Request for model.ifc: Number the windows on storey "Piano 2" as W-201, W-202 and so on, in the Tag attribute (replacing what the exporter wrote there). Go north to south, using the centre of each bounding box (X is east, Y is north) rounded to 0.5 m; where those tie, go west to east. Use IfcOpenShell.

First a look at what the model holds.

```python
import ifcopenshell
import ifcopenshell.util.element
import ifcopenshell.util.placement

model = ifcopenshell.open("model.ifc")
print(model.schema)
storey = next(s for s in model.by_type("IfcBuildingStorey") if s.Name == "Piano 2")
windows = [e for e in ifcopenshell.util.element.get_decomposition(storey) if e.is_a("IfcWindow")]
for e in sorted(windows, key=lambda e: e.id()):
    origin = ifcopenshell.util.placement.get_local_placement(e.ObjectPlacement)[:3, 3]
    print(e.id(), e.Tag, e.Name, origin.round(2) + 0.0, sep=" | ")
```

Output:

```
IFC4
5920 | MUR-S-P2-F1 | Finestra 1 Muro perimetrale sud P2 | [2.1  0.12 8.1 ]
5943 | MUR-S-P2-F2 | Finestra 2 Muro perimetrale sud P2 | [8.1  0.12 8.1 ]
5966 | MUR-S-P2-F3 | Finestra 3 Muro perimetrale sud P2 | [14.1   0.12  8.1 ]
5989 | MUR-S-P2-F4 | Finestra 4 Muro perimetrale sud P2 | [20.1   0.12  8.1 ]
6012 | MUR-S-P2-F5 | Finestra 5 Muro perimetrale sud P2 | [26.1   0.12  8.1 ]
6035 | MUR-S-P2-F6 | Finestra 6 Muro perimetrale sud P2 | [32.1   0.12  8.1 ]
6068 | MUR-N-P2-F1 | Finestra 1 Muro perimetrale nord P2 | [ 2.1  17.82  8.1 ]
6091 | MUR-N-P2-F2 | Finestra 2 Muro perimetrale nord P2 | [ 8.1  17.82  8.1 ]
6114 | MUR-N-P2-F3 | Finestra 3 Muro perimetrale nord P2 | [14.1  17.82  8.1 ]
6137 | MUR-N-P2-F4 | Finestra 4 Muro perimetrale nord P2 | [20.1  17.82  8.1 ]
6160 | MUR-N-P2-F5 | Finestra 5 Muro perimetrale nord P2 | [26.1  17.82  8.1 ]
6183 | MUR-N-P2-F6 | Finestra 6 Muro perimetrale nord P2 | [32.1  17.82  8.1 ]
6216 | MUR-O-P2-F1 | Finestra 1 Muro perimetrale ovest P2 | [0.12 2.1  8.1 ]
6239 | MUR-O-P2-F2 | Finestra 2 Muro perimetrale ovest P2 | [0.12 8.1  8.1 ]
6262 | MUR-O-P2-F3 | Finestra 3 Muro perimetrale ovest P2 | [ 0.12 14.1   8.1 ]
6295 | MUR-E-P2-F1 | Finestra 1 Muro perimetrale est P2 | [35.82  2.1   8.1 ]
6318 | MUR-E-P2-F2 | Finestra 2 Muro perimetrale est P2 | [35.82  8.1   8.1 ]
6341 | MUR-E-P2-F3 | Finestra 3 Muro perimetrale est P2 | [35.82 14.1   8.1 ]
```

```python
import ifcopenshell
import ifcopenshell.geom
import ifcopenshell.util.element
import ifcopenshell.util.shape

model = ifcopenshell.open("model.ifc")
settings = ifcopenshell.geom.settings()
settings.set("use-world-coords", True)


def centre(element):
    shape = ifcopenshell.geom.create_shape(settings, element)
    return ifcopenshell.util.shape.get_bbox_centroid(shape.geometry)


storey = next(s for s in model.by_type("IfcBuildingStorey") if s.Name == "Piano 2")
windows = [e for e in ifcopenshell.util.element.get_decomposition(storey) if e.is_a("IfcWindow")]

# Insertion points can sit at a corner or the storey origin, so sort by the geometry (in metres).
centres = {e: centre(e) for e in windows}
windows.sort(key=lambda e: (-round(centres[e][1] / 0.5), centres[e][0]))

for i, e in enumerate(windows, start=1):
    number = f"W-2{i:02d}"
    e.Tag = number
    print(e.id(), number)

model.write("model_v2.ifc")
```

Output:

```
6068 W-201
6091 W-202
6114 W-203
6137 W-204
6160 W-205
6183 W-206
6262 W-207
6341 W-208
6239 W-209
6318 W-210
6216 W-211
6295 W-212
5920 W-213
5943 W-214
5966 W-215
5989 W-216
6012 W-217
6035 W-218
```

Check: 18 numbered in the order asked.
